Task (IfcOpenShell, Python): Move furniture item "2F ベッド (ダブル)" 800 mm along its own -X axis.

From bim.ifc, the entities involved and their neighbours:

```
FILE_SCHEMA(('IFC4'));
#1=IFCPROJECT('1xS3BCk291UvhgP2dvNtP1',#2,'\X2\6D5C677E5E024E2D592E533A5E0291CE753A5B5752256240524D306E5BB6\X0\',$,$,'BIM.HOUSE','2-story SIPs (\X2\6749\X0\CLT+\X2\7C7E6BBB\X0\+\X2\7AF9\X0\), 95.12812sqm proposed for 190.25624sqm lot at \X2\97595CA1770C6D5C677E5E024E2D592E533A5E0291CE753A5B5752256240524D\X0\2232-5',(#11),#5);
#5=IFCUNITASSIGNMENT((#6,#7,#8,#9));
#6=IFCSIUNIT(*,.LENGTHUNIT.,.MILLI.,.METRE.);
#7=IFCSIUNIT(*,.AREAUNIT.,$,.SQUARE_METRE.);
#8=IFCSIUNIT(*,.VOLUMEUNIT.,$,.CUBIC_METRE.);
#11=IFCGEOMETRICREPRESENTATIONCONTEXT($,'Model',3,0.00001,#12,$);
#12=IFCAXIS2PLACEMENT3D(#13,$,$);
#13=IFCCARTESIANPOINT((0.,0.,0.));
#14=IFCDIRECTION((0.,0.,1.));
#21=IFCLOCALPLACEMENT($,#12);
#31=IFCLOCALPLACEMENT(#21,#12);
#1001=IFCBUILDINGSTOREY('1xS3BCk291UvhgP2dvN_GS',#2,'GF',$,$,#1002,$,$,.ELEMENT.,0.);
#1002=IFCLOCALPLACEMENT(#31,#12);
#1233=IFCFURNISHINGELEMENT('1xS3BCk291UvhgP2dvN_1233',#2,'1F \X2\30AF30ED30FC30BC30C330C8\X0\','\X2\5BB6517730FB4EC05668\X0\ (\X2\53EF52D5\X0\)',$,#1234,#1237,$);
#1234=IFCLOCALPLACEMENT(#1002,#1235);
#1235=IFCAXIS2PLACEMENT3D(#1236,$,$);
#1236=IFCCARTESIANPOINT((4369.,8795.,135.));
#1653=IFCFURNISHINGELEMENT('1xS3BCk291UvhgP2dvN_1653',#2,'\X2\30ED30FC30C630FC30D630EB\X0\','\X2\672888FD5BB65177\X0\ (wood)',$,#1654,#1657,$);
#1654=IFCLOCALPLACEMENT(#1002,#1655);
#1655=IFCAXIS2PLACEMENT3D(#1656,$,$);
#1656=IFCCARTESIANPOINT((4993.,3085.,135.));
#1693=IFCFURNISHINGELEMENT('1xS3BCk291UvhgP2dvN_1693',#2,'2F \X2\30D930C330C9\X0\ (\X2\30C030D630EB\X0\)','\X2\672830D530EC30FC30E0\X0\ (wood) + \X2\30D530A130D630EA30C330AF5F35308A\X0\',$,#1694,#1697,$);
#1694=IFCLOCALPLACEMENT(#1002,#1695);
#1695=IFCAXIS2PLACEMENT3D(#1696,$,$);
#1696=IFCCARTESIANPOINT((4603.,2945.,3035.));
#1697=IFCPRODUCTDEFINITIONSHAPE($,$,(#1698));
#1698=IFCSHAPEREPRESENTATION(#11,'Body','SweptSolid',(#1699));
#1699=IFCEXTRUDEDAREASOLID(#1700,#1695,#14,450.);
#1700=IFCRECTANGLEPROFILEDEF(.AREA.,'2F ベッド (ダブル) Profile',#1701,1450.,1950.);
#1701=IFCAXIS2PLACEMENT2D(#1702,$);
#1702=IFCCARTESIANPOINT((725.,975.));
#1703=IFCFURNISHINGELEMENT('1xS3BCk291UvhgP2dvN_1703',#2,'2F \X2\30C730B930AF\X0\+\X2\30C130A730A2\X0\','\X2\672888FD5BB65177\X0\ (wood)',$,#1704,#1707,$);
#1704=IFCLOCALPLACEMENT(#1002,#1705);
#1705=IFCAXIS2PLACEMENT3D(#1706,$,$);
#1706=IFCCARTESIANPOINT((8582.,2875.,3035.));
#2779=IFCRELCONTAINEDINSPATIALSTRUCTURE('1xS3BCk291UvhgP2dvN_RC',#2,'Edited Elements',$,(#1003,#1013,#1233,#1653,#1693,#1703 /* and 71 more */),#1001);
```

```python
import ifcopenshell
import ifcopenshell.api.geometry
import ifcopenshell.util.placement
import ifcopenshell.util.unit

model = ifcopenshell.open("bim.ifc")
unit_scale = ifcopenshell.util.unit.calculate_unit_scale(model)

item = model.by_guid("1xS3BCk291UvhgP2dvN_1693")
matrix = ifcopenshell.util.placement.get_local_placement(item.ObjectPlacement)
matrix[:3, 3] -= matrix[:3, 0] * 0.8 / unit_scale
ifcopenshell.api.geometry.edit_object_placement(model, product=item, matrix=matrix, is_si=False)

print(ifcopenshell.util.placement.get_local_placement(item.ObjectPlacement).round(3) + 0.0)

model.write("bim_v2.ifc")
```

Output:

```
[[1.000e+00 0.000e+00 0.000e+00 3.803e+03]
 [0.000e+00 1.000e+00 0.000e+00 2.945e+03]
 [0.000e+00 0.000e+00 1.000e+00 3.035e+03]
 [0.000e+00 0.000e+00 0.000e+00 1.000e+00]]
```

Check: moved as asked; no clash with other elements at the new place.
